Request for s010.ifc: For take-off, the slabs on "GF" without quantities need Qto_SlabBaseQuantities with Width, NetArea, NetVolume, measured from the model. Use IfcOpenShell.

First a look at what the model holds.

```python
import ifcopenshell
import ifcopenshell.util.element
import ifcopenshell.util.unit

model = ifcopenshell.open("s010.ifc")
print(model.schema)
for unit_type in ("LENGTHUNIT", "AREAUNIT", "VOLUMEUNIT"):
    print(unit_type, ifcopenshell.util.unit.calculate_unit_scale(model, unit_type))
storey = next(s for s in model.by_type("IfcBuildingStorey") if s.Name == "GF")
slabs = [e for e in ifcopenshell.util.element.get_decomposition(storey) if e.is_a("IfcSlab")]
for e in sorted(slabs, key=lambda e: e.id()):
    print(e.id(), e.is_a(), e.Name, list(ifcopenshell.util.element.get_psets(e, qtos_only=True)), sep=" | ")
```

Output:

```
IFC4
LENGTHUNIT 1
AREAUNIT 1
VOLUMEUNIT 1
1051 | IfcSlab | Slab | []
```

```python
import ifcopenshell
import ifcopenshell.api.pset
import ifcopenshell.geom
import ifcopenshell.util.element
import ifcopenshell.util.shape
import ifcopenshell.util.unit

model = ifcopenshell.open("s010.ifc")
unit_scale = ifcopenshell.util.unit.calculate_unit_scale(model)
area_scale = ifcopenshell.util.unit.calculate_unit_scale(model, "AREAUNIT")
volume_scale = ifcopenshell.util.unit.calculate_unit_scale(model, "VOLUMEUNIT")
settings = ifcopenshell.geom.settings()

storey = next(s for s in model.by_type("IfcBuildingStorey") if s.Name == "GF")
slabs = [e for e in ifcopenshell.util.element.get_decomposition(storey) if e.is_a("IfcSlab")]

for e in sorted(slabs, key=lambda e: e.id()):
    if ifcopenshell.util.element.get_psets(e, qtos_only=True, should_inherit=False):
        continue
    # Geometry comes back in metres, in the element's own axes.
    shape = ifcopenshell.geom.create_shape(settings, e)
    values = {
        "Width": ifcopenshell.util.shape.get_z(shape.geometry) / unit_scale,
        "NetArea": ifcopenshell.util.shape.get_footprint_area(shape.geometry) / area_scale,
        "NetVolume": ifcopenshell.util.shape.get_volume(shape.geometry) / volume_scale,
    }
    qto = ifcopenshell.api.pset.add_qto(model, product=e, name="Qto_SlabBaseQuantities")
    ifcopenshell.api.pset.edit_qto(model, qto=qto, properties=values)
    print(e.id(), {k: round(v, 3) for k, v in values.items()})

model.write("s010_updated.ifc")
```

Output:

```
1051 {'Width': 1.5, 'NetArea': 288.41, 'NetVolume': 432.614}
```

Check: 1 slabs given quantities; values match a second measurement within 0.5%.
